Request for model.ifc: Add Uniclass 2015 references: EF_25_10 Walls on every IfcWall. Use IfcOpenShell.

First a look at what the model holds.

```python
import ifcopenshell

model = ifcopenshell.open("model.ifc")
print(model.schema)
print("classifications:", [c.Name for c in model.by_type("IfcClassification")])
for ifc_class in ("IfcDoor", "IfcRoof", "IfcStair", "IfcWall", "IfcWindow"):
    print(ifc_class, len(model.by_type(ifc_class)))
```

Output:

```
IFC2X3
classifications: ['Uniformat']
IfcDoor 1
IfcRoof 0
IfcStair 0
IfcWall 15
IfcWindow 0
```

```python
import ifcopenshell
import ifcopenshell.api.classification

model = ifcopenshell.open("model.ifc")

# IFC2X3 requires Source and Edition and has no link from the project to the system.
system = model.create_entity("IfcClassification", Source="NBS", Edition="2015", Name="Uniclass 2015")

codes = {
    "IfcWall": ("EF_25_10", "Walls"),
}
for ifc_class, (code, name) in codes.items():
    products = model.by_type(ifc_class)
    ifcopenshell.api.classification.add_reference(
        model, products=products, classification=system, identification=code, name=name
    )
    print(code, len(products))

model.write("model-out.ifc")
```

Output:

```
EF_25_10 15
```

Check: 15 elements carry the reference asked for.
